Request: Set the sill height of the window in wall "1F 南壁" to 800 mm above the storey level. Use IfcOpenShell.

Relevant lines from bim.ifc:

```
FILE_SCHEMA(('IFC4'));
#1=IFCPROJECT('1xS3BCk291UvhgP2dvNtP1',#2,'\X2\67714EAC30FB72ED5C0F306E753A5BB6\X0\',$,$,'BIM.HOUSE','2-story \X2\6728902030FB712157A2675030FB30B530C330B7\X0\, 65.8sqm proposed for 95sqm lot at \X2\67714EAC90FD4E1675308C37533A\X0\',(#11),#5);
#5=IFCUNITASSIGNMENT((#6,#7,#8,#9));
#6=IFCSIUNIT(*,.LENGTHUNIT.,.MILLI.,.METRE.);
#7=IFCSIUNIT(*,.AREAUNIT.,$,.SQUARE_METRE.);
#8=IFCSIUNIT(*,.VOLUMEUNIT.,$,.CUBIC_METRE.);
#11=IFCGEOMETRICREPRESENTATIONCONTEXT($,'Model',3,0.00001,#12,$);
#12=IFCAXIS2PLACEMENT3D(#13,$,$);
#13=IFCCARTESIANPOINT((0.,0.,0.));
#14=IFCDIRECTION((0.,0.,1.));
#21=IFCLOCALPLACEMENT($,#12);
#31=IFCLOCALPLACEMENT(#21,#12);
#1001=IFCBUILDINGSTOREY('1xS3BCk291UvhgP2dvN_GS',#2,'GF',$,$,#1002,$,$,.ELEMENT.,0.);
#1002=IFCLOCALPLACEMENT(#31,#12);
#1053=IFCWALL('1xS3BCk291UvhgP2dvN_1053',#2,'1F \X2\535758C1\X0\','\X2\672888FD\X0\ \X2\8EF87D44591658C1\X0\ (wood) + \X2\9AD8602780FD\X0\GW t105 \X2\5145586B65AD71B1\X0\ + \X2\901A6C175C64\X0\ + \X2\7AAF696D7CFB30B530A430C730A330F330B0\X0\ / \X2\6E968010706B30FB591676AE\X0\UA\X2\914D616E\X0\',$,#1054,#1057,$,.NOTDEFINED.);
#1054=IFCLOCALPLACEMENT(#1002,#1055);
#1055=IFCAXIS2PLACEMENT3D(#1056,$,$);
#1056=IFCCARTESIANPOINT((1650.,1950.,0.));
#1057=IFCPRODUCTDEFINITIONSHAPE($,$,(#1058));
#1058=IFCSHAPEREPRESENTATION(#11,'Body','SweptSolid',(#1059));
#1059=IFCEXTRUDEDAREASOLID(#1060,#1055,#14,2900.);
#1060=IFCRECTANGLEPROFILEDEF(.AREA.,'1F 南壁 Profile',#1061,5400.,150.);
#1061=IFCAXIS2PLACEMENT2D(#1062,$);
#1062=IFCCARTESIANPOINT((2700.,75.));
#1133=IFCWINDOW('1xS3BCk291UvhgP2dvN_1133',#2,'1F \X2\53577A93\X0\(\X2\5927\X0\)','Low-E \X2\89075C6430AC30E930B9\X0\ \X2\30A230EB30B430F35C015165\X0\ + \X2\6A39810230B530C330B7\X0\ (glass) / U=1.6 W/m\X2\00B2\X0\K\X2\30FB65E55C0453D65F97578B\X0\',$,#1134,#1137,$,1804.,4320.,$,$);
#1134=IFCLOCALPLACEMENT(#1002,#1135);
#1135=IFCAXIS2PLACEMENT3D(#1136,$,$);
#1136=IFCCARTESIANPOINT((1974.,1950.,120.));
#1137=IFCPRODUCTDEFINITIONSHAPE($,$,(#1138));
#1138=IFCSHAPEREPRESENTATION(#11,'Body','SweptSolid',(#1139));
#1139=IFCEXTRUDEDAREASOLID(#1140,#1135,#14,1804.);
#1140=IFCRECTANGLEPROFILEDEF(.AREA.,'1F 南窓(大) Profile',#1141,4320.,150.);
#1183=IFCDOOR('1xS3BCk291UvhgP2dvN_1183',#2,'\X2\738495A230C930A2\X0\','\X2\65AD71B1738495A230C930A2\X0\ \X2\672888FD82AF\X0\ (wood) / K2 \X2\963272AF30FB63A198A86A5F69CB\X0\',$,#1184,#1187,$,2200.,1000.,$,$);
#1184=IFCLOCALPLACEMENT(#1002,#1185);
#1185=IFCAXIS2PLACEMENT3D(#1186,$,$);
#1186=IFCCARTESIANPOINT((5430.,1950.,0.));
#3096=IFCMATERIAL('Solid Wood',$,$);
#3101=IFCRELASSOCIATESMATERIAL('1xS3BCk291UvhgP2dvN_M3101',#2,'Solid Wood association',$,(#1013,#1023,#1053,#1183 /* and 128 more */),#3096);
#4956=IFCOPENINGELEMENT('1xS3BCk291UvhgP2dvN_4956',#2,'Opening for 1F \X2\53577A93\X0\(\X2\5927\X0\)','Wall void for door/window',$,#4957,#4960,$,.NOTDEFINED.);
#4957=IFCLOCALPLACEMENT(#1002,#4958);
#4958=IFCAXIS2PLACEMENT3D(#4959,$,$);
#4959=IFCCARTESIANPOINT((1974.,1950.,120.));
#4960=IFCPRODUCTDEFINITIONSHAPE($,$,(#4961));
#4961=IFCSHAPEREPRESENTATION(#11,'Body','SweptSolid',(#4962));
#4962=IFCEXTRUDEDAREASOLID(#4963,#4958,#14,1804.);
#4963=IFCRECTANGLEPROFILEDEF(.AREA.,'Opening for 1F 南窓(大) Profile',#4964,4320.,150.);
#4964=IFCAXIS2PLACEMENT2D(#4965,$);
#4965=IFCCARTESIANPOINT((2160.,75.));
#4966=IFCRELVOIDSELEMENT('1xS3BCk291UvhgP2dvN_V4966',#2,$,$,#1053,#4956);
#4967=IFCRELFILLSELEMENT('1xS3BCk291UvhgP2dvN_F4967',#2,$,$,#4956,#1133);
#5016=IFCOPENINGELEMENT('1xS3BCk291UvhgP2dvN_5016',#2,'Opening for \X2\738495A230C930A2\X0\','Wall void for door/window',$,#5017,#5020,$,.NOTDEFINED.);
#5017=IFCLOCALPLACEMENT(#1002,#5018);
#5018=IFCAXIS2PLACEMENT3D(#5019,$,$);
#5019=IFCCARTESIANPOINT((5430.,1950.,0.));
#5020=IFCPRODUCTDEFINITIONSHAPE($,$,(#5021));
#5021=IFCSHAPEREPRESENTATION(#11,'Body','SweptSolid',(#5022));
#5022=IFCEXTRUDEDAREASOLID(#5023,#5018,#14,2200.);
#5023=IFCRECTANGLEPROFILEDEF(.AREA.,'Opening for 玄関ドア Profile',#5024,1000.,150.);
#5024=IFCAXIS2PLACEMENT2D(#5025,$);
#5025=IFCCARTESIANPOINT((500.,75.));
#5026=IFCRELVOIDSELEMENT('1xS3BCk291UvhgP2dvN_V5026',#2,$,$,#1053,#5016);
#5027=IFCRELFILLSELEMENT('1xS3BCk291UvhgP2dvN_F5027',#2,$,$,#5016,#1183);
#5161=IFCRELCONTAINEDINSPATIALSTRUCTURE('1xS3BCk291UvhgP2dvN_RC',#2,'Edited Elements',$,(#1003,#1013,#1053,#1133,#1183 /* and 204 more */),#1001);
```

```python
import numpy as np
import ifcopenshell
import ifcopenshell.api.geometry
import ifcopenshell.geom
import ifcopenshell.util.element
import ifcopenshell.util.placement
import ifcopenshell.util.shape
import ifcopenshell.util.unit

model = ifcopenshell.open("bim.ifc")
unit_scale = ifcopenshell.util.unit.calculate_unit_scale(model)

window = model.by_id(1133)
opening = window.FillsVoids[0].RelatingOpeningElement
storey = ifcopenshell.util.element.get_container(window, ifc_class="IfcBuildingStorey")
level = ifcopenshell.util.placement.get_local_placement(storey.ObjectPlacement)[2, 3]

# The opening's origin need not be at the sill, so measure its lowest point.
shape = ifcopenshell.geom.create_shape(ifcopenshell.geom.settings(), opening)
bottom = ifcopenshell.util.shape.get_shape_bottom_elevation(shape, shape.geometry) / unit_scale
dz = level + 0.8 / unit_scale - bottom

shift = np.array([0.0, 0.0, dz])
# The window is not placed relative to its opening, so move both.
for product in (opening, window):
    matrix = ifcopenshell.util.placement.get_local_placement(product.ObjectPlacement)
    matrix[:3, 3] += shift
    ifcopenshell.api.geometry.edit_object_placement(model, product=product, matrix=matrix, is_si=False)

print(f"moved by {dz * unit_scale:+.3f} m")

model.write("bim_updated.ifc")
```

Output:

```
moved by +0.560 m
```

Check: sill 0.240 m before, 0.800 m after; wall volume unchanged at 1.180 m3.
